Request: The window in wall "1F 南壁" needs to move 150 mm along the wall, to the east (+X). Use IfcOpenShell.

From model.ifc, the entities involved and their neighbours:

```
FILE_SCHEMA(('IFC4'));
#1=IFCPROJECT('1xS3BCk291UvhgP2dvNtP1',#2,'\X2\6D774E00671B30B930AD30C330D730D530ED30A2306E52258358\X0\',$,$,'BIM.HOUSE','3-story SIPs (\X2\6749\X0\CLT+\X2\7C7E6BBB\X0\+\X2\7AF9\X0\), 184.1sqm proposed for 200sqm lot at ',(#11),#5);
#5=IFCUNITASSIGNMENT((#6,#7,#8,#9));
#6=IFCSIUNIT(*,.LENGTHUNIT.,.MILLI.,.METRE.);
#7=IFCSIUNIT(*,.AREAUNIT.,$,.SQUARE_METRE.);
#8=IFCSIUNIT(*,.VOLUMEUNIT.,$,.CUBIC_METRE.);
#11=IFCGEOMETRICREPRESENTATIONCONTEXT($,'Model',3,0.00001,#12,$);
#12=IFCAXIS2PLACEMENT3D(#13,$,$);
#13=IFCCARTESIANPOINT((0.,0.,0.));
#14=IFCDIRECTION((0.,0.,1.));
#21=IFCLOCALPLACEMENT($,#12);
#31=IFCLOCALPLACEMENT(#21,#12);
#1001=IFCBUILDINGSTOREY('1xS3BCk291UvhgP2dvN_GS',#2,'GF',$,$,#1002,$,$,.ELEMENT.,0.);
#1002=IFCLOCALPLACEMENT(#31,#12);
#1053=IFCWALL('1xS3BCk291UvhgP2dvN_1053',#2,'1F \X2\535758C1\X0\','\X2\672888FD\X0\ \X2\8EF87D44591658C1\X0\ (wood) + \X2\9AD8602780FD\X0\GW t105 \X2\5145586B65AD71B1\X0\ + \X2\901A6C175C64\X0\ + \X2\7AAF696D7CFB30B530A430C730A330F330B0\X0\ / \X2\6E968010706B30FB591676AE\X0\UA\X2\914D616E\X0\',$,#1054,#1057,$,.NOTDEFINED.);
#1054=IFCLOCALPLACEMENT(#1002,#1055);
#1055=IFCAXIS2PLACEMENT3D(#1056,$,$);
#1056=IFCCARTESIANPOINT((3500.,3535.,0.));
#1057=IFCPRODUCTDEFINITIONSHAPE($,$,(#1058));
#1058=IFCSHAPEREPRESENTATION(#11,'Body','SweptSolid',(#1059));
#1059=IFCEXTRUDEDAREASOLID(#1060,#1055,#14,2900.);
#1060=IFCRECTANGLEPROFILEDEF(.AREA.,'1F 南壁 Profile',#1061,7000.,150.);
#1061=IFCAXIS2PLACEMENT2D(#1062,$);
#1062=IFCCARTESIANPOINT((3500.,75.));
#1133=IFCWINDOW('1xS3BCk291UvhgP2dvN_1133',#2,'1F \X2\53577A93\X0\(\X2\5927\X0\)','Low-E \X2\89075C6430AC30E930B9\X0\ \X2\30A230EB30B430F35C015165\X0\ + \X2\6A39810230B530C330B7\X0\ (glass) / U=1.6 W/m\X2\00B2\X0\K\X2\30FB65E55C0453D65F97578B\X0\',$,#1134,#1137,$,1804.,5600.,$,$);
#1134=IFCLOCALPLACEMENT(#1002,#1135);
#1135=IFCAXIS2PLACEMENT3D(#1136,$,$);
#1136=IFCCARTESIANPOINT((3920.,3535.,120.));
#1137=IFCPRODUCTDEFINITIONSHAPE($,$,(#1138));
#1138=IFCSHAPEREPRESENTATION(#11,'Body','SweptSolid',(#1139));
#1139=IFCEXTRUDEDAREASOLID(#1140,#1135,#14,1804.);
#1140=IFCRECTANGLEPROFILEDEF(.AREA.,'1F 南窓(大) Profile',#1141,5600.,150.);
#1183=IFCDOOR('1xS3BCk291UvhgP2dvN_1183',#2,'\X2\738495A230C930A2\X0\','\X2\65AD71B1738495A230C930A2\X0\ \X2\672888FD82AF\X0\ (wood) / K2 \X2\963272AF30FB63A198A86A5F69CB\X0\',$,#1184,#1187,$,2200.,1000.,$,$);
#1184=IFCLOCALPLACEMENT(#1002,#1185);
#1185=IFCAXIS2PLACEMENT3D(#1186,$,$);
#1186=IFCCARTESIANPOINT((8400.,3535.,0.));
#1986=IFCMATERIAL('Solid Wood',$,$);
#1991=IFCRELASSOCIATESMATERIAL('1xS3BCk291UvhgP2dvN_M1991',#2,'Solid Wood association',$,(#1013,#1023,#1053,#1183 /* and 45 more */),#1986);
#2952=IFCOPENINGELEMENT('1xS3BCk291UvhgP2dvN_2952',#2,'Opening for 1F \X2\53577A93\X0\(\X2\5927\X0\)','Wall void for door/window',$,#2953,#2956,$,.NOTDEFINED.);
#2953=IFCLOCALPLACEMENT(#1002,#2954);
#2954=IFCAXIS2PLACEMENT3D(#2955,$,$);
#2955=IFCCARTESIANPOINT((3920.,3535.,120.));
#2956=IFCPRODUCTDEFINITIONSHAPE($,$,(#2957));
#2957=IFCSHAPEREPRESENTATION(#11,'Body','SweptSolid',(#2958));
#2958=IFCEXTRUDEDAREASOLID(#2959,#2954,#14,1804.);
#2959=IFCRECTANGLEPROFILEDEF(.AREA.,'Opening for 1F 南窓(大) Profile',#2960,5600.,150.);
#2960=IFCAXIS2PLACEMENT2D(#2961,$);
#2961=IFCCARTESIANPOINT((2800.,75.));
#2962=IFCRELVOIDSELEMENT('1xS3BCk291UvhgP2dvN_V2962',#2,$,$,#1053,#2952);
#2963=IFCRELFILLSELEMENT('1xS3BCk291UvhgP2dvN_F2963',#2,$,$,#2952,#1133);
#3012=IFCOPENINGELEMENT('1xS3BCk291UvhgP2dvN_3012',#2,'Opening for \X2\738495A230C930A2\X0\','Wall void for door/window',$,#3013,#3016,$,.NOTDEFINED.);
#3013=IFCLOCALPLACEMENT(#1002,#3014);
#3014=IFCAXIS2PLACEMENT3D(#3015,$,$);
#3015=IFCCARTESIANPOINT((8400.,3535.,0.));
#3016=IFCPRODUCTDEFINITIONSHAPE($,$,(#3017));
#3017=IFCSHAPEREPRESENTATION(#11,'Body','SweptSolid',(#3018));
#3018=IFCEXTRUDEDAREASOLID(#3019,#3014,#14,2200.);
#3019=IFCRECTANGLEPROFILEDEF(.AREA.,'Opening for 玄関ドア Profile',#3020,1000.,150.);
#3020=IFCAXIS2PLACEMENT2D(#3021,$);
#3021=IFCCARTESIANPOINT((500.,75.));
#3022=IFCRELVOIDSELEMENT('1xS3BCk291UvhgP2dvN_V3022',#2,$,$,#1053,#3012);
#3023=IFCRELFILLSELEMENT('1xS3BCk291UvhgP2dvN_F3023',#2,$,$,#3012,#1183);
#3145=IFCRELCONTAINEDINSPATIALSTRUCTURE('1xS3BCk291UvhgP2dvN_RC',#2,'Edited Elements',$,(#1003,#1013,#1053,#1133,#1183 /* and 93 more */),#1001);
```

```python
import ifcopenshell
import ifcopenshell.api.geometry
import ifcopenshell.util.placement

model = ifcopenshell.open("model.ifc")

window = model.by_id(1133)
opening = window.FillsVoids[0].RelatingOpeningElement
wall = opening.VoidsElements[0].RelatingBuildingElement

wall_matrix = ifcopenshell.util.placement.get_local_placement(wall.ObjectPlacement)
shift = wall_matrix[:3, 0] * 150.0
before = ifcopenshell.util.placement.get_local_placement(window.ObjectPlacement)[:3, 3].copy()

# The window is not placed relative to its opening, so move both.
for product in (opening, window):
    matrix = ifcopenshell.util.placement.get_local_placement(product.ObjectPlacement)
    matrix[:3, 3] += shift
    ifcopenshell.api.geometry.edit_object_placement(model, product=product, matrix=matrix, is_si=False)

after = ifcopenshell.util.placement.get_local_placement(window.ObjectPlacement)[:3, 3]
print("window moved by", (after - before).round(3) + 0.0)

model.write("model_edited.ifc")
```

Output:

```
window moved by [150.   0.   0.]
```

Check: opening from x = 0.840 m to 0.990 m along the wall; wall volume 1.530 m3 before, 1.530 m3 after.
